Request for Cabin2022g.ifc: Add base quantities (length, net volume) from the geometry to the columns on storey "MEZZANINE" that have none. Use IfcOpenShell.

First a look at what the model holds.

```python
import ifcopenshell
import ifcopenshell.util.element
import ifcopenshell.util.unit

model = ifcopenshell.open("Cabin2022g.ifc")
print(model.schema)
for unit_type in ("LENGTHUNIT", "AREAUNIT", "VOLUMEUNIT"):
    print(unit_type, ifcopenshell.util.unit.calculate_unit_scale(model, unit_type))
storey = next(s for s in model.by_type("IfcBuildingStorey") if s.Name == "MEZZANINE")
columns = [e for e in ifcopenshell.util.element.get_decomposition(storey) if e.is_a("IfcColumn")]
for e in sorted(columns, key=lambda e: e.id()):
    print(e.id(), e.is_a(), e.Name, list(ifcopenshell.util.element.get_psets(e, qtos_only=True)), sep=" | ")
```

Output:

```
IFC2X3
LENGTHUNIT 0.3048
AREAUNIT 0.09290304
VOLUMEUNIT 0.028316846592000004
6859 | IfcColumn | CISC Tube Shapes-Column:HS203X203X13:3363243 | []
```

```python
import ifcopenshell
import ifcopenshell.api.pset
import ifcopenshell.geom
import ifcopenshell.util.element
import ifcopenshell.util.shape
import ifcopenshell.util.unit

model = ifcopenshell.open("Cabin2022g.ifc")
unit_scale = ifcopenshell.util.unit.calculate_unit_scale(model)
volume_scale = ifcopenshell.util.unit.calculate_unit_scale(model, "VOLUMEUNIT")
settings = ifcopenshell.geom.settings()

storey = next(s for s in model.by_type("IfcBuildingStorey") if s.Name == "MEZZANINE")
columns = [e for e in ifcopenshell.util.element.get_decomposition(storey) if e.is_a("IfcColumn")]

for e in sorted(columns, key=lambda e: e.id()):
    if ifcopenshell.util.element.get_psets(e, qtos_only=True, should_inherit=False):
        continue
    # Geometry comes back in metres, in the element's own axes.
    shape = ifcopenshell.geom.create_shape(settings, e)
    values = {
        "Length": ifcopenshell.util.shape.get_z(shape.geometry) / unit_scale,
        "NetVolume": ifcopenshell.util.shape.get_volume(shape.geometry) / volume_scale,
    }
    qto = ifcopenshell.api.pset.add_qto(model, product=e, name="BaseQuantities")
    ifcopenshell.api.pset.edit_qto(model, qto=qto, properties=values)
    print(e.id(), {k: round(v, 3) for k, v in values.items()})

model.write("Cabin2022g_v2.ifc")
```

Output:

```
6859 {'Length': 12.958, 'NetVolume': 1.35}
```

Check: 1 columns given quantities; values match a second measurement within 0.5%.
